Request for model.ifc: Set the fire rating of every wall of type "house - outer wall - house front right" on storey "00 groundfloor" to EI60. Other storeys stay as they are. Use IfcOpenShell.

First a look at what the model holds.

```python
import ifcopenshell
import ifcopenshell.util.element

model = ifcopenshell.open("model.ifc")
print(model.schema)
storey = next(s for s in model.by_type("IfcBuildingStorey") if s.Name == "00 groundfloor")
walls = [e for e in ifcopenshell.util.element.get_decomposition(storey) if e.is_a("IfcWall")]
seen = {}
for e in walls:
    element_type = ifcopenshell.util.element.get_type(e)
    key = (element_type.Name if element_type != e and element_type else None, ifcopenshell.util.element.get_pset(e, "Pset_WallCommon", "FireRating"))
    seen[key] = seen.get(key, 0) + 1
for (name, value), count in sorted(seen.items(), key=str):
    print(count, "x", name, "|", value)
```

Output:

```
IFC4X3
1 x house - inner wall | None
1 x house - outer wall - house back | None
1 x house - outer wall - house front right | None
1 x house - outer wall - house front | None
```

```python
import ifcopenshell
import ifcopenshell.api.pset
import ifcopenshell.util.element

model = ifcopenshell.open("model.ifc")

storey = next(s for s in model.by_type("IfcBuildingStorey") if s.Name == "00 groundfloor")
walls = [e for e in ifcopenshell.util.element.get_decomposition(storey) if e.is_a("IfcWall")]

count = 0
for e in walls:
    element_type = ifcopenshell.util.element.get_type(e)
    if element_type in (None, e) or element_type.Name != "house - outer wall - house front right":
        continue
    # add_pset returns the element's existing set when there is one.
    pset = ifcopenshell.api.pset.add_pset(model, product=e, name="Pset_WallCommon")
    ifcopenshell.api.pset.edit_pset(model, pset=pset, properties={"FireRating": "EI60"})
    count += 1

print(count, "walls updated")

model.write("model_updated.ifc")
```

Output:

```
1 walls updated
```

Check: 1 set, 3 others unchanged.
